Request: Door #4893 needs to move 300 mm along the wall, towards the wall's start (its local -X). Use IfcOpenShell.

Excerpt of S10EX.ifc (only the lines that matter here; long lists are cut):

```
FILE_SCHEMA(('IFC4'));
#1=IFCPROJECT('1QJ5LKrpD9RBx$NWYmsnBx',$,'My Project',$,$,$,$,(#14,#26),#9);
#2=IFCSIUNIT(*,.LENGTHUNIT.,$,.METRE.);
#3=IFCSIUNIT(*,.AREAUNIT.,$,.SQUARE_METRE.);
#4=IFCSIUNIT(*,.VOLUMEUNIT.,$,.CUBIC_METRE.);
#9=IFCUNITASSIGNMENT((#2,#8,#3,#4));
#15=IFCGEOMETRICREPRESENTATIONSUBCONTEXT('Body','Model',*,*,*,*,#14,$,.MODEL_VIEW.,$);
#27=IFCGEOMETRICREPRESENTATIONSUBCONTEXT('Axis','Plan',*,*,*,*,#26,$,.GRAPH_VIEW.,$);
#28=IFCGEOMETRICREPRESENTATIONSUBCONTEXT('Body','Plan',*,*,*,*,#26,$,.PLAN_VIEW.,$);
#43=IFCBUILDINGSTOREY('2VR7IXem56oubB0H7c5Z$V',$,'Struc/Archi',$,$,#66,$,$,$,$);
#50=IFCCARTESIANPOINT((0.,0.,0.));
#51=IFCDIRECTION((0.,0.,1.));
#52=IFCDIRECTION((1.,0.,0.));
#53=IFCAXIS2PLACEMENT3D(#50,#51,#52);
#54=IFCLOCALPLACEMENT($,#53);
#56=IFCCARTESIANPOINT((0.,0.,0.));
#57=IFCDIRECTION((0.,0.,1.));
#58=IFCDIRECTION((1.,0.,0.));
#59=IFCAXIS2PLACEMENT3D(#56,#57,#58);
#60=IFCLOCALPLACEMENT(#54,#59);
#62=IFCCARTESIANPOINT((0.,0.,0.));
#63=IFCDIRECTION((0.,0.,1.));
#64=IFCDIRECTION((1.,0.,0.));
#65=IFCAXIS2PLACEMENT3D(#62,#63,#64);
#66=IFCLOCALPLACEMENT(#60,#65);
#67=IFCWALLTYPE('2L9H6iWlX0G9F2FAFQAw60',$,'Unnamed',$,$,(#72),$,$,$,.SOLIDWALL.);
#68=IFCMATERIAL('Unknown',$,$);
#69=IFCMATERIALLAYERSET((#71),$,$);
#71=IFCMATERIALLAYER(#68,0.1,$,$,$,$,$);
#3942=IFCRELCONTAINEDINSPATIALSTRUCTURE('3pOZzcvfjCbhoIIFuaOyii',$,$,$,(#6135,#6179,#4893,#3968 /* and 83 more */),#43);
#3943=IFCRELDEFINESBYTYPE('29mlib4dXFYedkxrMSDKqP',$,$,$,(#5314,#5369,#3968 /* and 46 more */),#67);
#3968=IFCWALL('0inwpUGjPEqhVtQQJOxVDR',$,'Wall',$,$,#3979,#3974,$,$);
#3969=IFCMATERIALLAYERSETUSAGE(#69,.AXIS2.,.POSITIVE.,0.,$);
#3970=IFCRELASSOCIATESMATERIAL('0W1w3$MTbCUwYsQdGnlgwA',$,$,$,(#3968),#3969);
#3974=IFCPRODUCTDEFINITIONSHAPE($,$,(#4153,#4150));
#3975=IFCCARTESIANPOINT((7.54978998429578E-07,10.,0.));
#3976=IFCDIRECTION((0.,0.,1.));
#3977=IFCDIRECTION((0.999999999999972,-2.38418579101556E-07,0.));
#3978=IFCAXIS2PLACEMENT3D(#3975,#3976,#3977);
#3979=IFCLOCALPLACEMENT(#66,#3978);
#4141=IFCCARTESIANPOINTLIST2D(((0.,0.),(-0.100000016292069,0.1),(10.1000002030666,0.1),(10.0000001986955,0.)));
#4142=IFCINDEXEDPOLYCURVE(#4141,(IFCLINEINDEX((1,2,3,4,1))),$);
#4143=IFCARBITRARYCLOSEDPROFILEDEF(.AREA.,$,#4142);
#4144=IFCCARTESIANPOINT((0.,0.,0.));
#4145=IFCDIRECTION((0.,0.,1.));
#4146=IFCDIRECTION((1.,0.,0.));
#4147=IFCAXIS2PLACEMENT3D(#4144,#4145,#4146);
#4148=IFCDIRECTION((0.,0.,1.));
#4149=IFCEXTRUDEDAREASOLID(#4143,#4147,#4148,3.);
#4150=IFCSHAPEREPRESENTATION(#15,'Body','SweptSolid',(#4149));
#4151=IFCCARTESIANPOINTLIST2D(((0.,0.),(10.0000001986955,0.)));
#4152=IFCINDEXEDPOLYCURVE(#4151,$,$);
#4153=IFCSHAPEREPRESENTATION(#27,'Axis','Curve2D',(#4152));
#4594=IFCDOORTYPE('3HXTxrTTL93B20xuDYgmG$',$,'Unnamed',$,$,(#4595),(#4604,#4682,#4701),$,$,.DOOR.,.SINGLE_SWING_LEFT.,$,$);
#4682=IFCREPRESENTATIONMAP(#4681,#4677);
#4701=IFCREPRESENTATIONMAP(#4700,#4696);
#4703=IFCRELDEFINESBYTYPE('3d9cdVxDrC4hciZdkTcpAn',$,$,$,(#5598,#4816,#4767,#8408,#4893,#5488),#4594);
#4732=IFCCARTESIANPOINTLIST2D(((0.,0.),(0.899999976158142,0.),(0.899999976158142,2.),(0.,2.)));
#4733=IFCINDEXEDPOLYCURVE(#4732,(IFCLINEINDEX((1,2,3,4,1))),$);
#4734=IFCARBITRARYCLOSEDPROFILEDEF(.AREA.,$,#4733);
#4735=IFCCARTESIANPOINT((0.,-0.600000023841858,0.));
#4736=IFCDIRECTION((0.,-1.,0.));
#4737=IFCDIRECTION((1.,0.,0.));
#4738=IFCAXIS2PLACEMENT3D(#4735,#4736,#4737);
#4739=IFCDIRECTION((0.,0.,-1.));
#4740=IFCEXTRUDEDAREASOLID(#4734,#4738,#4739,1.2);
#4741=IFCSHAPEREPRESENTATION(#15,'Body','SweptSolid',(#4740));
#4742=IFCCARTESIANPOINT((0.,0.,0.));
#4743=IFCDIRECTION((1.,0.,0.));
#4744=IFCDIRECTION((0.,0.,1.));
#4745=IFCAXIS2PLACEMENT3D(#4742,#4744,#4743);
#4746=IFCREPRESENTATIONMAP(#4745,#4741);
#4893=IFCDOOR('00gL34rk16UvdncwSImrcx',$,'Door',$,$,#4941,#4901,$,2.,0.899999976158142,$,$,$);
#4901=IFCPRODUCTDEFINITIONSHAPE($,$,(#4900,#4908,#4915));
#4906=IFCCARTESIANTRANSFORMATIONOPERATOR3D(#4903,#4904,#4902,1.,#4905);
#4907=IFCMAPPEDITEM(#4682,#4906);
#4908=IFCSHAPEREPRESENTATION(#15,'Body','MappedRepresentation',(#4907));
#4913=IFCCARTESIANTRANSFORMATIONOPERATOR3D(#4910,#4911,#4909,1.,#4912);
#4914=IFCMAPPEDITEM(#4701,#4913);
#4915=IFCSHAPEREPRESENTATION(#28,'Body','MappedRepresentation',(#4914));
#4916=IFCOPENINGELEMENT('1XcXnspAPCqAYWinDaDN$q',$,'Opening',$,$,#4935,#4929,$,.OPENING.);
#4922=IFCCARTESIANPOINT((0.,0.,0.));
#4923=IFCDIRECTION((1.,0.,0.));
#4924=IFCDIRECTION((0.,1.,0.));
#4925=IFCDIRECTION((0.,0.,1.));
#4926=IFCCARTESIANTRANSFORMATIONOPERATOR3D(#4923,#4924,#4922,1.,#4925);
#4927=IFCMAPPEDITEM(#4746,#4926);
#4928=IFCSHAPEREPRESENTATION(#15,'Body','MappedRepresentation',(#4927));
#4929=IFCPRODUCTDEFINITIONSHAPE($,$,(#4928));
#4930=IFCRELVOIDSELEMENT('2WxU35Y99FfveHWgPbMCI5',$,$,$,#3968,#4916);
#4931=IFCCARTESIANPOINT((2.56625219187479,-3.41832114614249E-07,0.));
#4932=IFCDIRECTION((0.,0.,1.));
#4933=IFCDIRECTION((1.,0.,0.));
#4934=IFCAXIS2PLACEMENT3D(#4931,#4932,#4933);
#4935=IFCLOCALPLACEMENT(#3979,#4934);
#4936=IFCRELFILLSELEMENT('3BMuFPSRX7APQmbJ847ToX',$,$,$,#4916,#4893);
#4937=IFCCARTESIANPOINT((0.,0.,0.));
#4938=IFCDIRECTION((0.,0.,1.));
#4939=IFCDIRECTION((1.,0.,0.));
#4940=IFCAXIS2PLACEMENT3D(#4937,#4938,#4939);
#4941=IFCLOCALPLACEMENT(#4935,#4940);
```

```python
import ifcopenshell
import ifcopenshell.api.geometry
import ifcopenshell.util.placement
import ifcopenshell.util.unit

model = ifcopenshell.open("S10EX.ifc")
unit_scale = ifcopenshell.util.unit.calculate_unit_scale(model)

door = model.by_guid("00gL34rk16UvdncwSImrcx")
opening = door.FillsVoids[0].RelatingOpeningElement
wall = opening.VoidsElements[0].RelatingBuildingElement

wall_matrix = ifcopenshell.util.placement.get_local_placement(wall.ObjectPlacement)
shift = wall_matrix[:3, 0] * -0.3 / unit_scale
before = ifcopenshell.util.placement.get_local_placement(door.ObjectPlacement)[:3, 3].copy()

# The door is placed relative to its opening, so it follows when the opening moves.
matrix = ifcopenshell.util.placement.get_local_placement(opening.ObjectPlacement)
matrix[:3, 3] += shift
ifcopenshell.api.geometry.edit_object_placement(
    model, product=opening, matrix=matrix, is_si=False, should_transform_children=True
)

after = ifcopenshell.util.placement.get_local_placement(door.ObjectPlacement)[:3, 3]
print("door moved by", (after - before).round(3) + 0.0)

model.write("S10EX-out.ifc")
```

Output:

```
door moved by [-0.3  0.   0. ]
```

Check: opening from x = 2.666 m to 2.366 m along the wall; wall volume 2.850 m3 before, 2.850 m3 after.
